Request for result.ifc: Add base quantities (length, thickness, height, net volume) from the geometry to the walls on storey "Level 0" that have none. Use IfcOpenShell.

First a look at what the model holds.

```python
import ifcopenshell
import ifcopenshell.util.element
import ifcopenshell.util.unit

model = ifcopenshell.open("result.ifc")
print(model.schema)
for unit_type in ("LENGTHUNIT", "AREAUNIT", "VOLUMEUNIT"):
    print(unit_type, ifcopenshell.util.unit.calculate_unit_scale(model, unit_type))
storey = next(s for s in model.by_type("IfcBuildingStorey") if s.Name == "Level 0")
walls = [e for e in ifcopenshell.util.element.get_decomposition(storey) if e.is_a("IfcWall")]
for e in sorted(walls, key=lambda e: e.id()):
    print(e.id(), e.is_a(), e.Name, list(ifcopenshell.util.element.get_psets(e, qtos_only=True)), sep=" | ")
```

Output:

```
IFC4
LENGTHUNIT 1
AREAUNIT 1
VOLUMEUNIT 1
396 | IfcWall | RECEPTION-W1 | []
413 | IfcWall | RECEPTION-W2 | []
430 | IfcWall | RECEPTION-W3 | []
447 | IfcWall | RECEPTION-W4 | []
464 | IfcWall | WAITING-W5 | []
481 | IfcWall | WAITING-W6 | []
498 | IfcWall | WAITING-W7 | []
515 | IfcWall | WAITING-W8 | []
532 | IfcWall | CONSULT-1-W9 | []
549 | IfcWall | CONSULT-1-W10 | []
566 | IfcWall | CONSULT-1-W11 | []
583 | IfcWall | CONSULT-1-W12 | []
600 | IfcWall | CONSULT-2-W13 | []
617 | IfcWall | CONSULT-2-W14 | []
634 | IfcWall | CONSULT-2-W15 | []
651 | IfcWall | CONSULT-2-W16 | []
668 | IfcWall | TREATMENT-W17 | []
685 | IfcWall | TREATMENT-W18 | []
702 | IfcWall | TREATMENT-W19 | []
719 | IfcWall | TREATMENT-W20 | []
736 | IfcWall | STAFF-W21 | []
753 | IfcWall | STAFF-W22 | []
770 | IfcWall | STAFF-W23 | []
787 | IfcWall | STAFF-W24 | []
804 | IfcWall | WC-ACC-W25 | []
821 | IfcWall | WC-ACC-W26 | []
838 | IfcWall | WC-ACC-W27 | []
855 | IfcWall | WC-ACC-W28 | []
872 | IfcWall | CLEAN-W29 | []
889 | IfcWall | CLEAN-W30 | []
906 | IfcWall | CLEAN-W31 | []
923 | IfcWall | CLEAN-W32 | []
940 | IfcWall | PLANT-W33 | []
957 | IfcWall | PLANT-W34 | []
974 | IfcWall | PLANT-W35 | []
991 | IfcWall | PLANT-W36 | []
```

```python
import ifcopenshell
import ifcopenshell.api.pset
import ifcopenshell.geom
import ifcopenshell.util.element
import ifcopenshell.util.shape
import ifcopenshell.util.unit

model = ifcopenshell.open("result.ifc")
unit_scale = ifcopenshell.util.unit.calculate_unit_scale(model)
volume_scale = ifcopenshell.util.unit.calculate_unit_scale(model, "VOLUMEUNIT")
settings = ifcopenshell.geom.settings()

storey = next(s for s in model.by_type("IfcBuildingStorey") if s.Name == "Level 0")
walls = [e for e in ifcopenshell.util.element.get_decomposition(storey) if e.is_a("IfcWall")]

for e in sorted(walls, key=lambda e: e.id()):
    if ifcopenshell.util.element.get_psets(e, qtos_only=True, should_inherit=False):
        continue
    # Geometry comes back in metres, in the element's own axes.
    shape = ifcopenshell.geom.create_shape(settings, e)
    values = {
        "Length": ifcopenshell.util.shape.get_x(shape.geometry) / unit_scale,
        "Width": ifcopenshell.util.shape.get_y(shape.geometry) / unit_scale,
        "Height": ifcopenshell.util.shape.get_z(shape.geometry) / unit_scale,
        "NetVolume": ifcopenshell.util.shape.get_volume(shape.geometry) / volume_scale,
    }
    qto = ifcopenshell.api.pset.add_qto(model, product=e, name="Qto_WallBaseQuantities")
    ifcopenshell.api.pset.edit_qto(model, qto=qto, properties=values)
    print(e.id(), {k: round(v, 3) for k, v in values.items()})

model.write("result_v2.ifc")
```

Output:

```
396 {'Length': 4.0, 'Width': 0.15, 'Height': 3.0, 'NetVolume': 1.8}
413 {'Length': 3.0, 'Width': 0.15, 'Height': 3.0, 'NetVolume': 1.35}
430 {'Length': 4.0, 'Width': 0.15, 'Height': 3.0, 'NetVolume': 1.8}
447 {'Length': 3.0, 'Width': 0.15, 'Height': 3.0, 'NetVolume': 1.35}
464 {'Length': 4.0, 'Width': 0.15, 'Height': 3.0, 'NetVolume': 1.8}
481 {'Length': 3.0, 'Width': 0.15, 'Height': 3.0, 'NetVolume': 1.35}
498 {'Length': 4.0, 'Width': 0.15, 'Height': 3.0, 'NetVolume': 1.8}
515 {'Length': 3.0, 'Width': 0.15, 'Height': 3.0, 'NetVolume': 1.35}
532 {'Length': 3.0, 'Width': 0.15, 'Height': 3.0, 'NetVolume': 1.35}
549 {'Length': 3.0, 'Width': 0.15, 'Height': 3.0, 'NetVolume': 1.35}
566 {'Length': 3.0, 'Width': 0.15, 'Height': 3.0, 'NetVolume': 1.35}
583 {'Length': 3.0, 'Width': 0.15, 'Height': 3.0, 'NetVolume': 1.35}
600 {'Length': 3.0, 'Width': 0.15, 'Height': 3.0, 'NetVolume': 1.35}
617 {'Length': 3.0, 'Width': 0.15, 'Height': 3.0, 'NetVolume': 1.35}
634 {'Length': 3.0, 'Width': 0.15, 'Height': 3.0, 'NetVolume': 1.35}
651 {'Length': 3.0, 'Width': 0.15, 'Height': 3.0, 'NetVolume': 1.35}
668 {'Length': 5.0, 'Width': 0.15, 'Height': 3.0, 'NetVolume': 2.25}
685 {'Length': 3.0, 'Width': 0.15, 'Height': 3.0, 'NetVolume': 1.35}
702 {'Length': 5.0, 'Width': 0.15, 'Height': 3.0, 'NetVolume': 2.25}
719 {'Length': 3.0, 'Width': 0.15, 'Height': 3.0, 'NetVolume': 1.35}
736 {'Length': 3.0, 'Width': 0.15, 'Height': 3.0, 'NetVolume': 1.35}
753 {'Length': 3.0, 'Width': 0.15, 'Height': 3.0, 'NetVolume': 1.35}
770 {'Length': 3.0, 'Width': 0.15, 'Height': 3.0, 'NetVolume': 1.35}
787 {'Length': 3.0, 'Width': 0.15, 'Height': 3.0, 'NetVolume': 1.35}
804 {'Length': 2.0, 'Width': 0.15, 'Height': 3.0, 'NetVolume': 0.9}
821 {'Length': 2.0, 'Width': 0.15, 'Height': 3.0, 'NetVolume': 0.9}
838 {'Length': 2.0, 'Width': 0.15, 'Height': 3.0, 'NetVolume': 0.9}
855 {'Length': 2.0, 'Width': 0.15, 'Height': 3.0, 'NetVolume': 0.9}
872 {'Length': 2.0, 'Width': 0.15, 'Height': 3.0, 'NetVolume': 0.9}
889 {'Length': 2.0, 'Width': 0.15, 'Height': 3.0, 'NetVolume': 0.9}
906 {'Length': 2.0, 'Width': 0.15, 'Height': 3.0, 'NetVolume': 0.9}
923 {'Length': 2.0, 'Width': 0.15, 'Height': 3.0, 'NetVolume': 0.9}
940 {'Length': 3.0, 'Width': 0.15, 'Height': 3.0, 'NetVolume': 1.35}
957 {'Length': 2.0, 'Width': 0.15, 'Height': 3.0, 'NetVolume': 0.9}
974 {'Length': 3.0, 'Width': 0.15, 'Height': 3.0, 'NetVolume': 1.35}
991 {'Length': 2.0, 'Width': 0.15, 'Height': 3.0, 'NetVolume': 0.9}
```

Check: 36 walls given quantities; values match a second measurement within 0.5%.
